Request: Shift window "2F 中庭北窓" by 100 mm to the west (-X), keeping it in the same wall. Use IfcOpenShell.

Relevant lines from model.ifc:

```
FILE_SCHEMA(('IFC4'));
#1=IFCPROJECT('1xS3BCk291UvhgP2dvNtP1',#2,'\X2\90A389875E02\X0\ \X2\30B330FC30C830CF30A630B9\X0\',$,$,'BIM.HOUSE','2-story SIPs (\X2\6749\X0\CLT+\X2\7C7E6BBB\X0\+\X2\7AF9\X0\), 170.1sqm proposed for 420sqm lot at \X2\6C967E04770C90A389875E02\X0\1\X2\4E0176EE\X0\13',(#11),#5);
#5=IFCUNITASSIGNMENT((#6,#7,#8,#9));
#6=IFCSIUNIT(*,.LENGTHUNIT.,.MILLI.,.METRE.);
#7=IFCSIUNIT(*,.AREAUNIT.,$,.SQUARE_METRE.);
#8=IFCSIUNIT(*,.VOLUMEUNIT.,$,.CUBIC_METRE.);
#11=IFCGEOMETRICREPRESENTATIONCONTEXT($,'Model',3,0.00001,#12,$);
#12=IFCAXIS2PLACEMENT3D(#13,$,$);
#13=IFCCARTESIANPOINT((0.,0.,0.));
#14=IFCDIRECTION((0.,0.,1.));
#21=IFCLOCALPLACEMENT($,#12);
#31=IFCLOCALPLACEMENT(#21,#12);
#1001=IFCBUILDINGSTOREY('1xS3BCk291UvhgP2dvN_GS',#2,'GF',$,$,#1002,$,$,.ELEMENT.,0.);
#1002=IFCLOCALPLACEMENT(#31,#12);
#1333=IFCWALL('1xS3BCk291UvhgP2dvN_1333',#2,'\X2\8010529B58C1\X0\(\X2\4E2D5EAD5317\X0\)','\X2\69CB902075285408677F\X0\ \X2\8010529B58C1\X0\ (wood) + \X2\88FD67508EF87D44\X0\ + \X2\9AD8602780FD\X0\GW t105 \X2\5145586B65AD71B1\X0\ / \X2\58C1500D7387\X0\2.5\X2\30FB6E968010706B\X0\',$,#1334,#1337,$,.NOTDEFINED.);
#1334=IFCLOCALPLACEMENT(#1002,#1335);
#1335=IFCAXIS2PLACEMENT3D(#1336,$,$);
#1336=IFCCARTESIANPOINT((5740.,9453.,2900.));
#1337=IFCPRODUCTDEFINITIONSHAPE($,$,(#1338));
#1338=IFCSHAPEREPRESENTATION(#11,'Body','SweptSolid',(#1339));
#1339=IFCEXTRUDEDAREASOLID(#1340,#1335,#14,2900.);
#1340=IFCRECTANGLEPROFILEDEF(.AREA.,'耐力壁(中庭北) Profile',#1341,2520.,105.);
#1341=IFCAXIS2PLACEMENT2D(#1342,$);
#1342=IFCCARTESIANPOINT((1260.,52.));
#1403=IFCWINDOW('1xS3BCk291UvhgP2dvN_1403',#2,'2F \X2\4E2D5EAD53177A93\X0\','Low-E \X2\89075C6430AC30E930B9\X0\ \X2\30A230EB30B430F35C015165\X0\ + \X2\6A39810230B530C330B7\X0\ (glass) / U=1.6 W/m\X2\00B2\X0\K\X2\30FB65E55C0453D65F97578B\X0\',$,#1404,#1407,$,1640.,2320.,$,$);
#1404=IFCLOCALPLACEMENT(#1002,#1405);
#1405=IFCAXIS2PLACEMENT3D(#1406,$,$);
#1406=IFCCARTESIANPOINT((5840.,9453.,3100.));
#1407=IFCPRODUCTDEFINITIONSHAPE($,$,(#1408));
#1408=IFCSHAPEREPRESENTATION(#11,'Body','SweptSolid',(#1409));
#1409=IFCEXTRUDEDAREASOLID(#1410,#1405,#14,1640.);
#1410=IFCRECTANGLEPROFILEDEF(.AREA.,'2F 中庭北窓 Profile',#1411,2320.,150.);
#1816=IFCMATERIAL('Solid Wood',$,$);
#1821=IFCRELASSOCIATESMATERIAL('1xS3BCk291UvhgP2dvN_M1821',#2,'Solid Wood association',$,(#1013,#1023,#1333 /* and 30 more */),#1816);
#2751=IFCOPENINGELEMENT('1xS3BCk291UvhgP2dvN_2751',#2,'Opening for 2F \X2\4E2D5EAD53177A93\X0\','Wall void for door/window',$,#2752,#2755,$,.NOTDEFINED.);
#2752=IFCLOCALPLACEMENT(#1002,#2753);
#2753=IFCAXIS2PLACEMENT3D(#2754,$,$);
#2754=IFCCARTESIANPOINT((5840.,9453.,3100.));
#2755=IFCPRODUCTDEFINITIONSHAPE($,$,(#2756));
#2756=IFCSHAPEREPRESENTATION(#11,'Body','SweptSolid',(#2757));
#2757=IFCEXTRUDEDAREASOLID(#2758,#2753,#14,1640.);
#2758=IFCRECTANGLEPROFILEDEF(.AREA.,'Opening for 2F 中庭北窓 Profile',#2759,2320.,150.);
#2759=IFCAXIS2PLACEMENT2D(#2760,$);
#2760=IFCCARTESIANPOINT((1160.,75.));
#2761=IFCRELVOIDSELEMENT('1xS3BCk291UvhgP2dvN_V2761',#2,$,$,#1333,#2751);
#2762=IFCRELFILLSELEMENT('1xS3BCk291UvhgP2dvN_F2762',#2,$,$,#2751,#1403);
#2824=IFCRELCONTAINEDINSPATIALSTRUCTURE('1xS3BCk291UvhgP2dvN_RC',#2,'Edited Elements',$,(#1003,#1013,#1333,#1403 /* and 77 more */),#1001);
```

```python
import ifcopenshell
import ifcopenshell.api.geometry
import ifcopenshell.util.placement

model = ifcopenshell.open("model.ifc")

window = model.by_guid("1xS3BCk291UvhgP2dvN_1403")
opening = window.FillsVoids[0].RelatingOpeningElement
wall = opening.VoidsElements[0].RelatingBuildingElement

wall_matrix = ifcopenshell.util.placement.get_local_placement(wall.ObjectPlacement)
shift = wall_matrix[:3, 0] * -100.0
before = ifcopenshell.util.placement.get_local_placement(window.ObjectPlacement)[:3, 3].copy()

# The window is not placed relative to its opening, so move both.
for product in (opening, window):
    matrix = ifcopenshell.util.placement.get_local_placement(product.ObjectPlacement)
    matrix[:3, 3] += shift
    ifcopenshell.api.geometry.edit_object_placement(model, product=product, matrix=matrix, is_si=False)

after = ifcopenshell.util.placement.get_local_placement(window.ObjectPlacement)[:3, 3]
print("window moved by", (after - before).round(3) + 0.0)

model.write("model_updated.ifc")
```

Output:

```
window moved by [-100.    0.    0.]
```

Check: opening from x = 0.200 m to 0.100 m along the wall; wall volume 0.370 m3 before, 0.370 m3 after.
